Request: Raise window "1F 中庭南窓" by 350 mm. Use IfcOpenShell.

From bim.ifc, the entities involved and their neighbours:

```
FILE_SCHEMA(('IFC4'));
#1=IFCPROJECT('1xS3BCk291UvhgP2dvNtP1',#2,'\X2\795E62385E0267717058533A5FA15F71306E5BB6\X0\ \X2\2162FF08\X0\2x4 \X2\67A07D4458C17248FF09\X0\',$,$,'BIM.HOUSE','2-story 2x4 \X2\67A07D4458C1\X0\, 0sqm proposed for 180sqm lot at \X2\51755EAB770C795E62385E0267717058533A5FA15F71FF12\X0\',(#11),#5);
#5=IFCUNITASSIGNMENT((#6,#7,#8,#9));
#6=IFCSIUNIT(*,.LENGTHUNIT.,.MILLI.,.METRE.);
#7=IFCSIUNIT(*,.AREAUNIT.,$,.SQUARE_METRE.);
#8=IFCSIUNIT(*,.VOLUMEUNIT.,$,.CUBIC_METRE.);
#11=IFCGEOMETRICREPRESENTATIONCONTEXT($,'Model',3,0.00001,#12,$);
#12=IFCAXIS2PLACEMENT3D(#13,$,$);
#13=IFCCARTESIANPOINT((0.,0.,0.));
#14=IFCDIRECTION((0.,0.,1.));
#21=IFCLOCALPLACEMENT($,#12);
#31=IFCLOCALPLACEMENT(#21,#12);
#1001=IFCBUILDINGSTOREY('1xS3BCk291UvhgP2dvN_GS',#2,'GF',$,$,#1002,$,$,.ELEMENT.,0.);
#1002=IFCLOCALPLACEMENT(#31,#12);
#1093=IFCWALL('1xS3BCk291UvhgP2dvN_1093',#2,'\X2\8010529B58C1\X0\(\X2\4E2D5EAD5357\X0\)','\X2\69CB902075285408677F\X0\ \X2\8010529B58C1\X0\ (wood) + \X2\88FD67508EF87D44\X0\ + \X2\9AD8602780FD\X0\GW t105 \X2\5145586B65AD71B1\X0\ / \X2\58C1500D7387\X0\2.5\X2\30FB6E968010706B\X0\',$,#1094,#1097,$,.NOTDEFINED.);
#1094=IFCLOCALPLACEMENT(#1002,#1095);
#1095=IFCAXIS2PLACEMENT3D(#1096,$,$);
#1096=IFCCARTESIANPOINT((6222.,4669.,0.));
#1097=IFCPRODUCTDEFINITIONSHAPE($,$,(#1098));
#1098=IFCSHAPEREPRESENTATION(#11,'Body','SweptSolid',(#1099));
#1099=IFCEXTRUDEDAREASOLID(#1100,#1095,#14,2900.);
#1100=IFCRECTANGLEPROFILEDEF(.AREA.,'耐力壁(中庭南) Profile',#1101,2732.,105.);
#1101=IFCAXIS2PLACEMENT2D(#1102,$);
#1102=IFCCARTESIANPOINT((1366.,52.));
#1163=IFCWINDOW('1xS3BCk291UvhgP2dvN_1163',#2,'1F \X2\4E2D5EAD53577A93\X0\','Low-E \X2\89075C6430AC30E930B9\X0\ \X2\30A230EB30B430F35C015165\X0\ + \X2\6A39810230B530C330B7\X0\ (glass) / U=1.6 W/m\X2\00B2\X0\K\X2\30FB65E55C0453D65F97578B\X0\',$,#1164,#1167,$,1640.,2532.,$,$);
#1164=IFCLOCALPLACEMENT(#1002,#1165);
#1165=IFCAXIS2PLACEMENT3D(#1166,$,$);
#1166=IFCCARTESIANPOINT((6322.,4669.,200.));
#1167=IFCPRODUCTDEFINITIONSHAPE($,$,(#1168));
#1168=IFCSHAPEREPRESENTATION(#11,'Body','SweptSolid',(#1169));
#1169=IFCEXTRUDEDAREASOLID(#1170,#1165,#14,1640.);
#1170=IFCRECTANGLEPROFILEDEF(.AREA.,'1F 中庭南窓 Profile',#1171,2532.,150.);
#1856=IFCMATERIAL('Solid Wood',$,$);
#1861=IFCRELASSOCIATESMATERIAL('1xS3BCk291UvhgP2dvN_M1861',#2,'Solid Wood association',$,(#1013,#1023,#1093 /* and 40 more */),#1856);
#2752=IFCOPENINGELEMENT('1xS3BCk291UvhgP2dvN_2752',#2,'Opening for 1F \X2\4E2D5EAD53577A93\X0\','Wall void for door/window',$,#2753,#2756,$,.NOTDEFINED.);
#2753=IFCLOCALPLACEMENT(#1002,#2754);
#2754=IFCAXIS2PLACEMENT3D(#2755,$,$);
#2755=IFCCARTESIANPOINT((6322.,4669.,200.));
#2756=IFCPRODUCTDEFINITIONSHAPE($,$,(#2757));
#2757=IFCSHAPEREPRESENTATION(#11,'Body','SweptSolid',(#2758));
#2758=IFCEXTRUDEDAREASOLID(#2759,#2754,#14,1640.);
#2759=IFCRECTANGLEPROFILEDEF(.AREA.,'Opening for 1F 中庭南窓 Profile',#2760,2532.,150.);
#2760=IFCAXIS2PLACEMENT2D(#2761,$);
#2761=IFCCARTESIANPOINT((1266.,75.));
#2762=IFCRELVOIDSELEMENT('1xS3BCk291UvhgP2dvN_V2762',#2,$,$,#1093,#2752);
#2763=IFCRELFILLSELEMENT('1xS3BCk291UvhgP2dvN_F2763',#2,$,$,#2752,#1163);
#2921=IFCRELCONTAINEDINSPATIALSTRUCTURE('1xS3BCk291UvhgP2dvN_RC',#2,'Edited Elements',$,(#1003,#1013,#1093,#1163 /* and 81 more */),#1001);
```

```python
import numpy as np
import ifcopenshell
import ifcopenshell.api.geometry
import ifcopenshell.util.placement
import ifcopenshell.util.unit

model = ifcopenshell.open("bim.ifc")
unit_scale = ifcopenshell.util.unit.calculate_unit_scale(model)

window = model.by_guid("1xS3BCk291UvhgP2dvN_1163")
opening = window.FillsVoids[0].RelatingOpeningElement
dz = 0.35 / unit_scale

shift = np.array([0.0, 0.0, dz])
# The window is not placed relative to its opening, so move both.
for product in (opening, window):
    matrix = ifcopenshell.util.placement.get_local_placement(product.ObjectPlacement)
    matrix[:3, 3] += shift
    ifcopenshell.api.geometry.edit_object_placement(model, product=product, matrix=matrix, is_si=False)

print(f"moved by {dz * unit_scale:+.3f} m")

model.write("bim_rev.ifc")
```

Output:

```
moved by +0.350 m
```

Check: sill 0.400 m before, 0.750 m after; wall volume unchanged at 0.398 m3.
